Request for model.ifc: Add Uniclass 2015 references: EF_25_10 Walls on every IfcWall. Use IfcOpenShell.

First a look at what the model holds.

```python
import ifcopenshell

model = ifcopenshell.open("model.ifc")
print(model.schema)
print("classifications:", [c.Name for c in model.by_type("IfcClassification")])
for ifc_class in ("IfcDoor", "IfcRoof", "IfcStair", "IfcWall", "IfcWindow"):
    print(ifc_class, len(model.by_type(ifc_class)))
```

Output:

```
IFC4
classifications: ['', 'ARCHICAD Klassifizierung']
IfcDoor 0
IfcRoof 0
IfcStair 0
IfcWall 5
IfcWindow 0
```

```python
import ifcopenshell
import ifcopenshell.api.classification

model = ifcopenshell.open("model.ifc")

system = ifcopenshell.api.classification.add_classification(model, classification="Uniclass 2015")

codes = {
    "IfcWall": ("EF_25_10", "Walls"),
}
for ifc_class, (code, name) in codes.items():
    products = model.by_type(ifc_class)
    ifcopenshell.api.classification.add_reference(
        model, products=products, classification=system, identification=code, name=name
    )
    print(code, len(products))

model.write("model_v2.ifc")
```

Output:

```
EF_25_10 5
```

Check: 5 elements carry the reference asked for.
